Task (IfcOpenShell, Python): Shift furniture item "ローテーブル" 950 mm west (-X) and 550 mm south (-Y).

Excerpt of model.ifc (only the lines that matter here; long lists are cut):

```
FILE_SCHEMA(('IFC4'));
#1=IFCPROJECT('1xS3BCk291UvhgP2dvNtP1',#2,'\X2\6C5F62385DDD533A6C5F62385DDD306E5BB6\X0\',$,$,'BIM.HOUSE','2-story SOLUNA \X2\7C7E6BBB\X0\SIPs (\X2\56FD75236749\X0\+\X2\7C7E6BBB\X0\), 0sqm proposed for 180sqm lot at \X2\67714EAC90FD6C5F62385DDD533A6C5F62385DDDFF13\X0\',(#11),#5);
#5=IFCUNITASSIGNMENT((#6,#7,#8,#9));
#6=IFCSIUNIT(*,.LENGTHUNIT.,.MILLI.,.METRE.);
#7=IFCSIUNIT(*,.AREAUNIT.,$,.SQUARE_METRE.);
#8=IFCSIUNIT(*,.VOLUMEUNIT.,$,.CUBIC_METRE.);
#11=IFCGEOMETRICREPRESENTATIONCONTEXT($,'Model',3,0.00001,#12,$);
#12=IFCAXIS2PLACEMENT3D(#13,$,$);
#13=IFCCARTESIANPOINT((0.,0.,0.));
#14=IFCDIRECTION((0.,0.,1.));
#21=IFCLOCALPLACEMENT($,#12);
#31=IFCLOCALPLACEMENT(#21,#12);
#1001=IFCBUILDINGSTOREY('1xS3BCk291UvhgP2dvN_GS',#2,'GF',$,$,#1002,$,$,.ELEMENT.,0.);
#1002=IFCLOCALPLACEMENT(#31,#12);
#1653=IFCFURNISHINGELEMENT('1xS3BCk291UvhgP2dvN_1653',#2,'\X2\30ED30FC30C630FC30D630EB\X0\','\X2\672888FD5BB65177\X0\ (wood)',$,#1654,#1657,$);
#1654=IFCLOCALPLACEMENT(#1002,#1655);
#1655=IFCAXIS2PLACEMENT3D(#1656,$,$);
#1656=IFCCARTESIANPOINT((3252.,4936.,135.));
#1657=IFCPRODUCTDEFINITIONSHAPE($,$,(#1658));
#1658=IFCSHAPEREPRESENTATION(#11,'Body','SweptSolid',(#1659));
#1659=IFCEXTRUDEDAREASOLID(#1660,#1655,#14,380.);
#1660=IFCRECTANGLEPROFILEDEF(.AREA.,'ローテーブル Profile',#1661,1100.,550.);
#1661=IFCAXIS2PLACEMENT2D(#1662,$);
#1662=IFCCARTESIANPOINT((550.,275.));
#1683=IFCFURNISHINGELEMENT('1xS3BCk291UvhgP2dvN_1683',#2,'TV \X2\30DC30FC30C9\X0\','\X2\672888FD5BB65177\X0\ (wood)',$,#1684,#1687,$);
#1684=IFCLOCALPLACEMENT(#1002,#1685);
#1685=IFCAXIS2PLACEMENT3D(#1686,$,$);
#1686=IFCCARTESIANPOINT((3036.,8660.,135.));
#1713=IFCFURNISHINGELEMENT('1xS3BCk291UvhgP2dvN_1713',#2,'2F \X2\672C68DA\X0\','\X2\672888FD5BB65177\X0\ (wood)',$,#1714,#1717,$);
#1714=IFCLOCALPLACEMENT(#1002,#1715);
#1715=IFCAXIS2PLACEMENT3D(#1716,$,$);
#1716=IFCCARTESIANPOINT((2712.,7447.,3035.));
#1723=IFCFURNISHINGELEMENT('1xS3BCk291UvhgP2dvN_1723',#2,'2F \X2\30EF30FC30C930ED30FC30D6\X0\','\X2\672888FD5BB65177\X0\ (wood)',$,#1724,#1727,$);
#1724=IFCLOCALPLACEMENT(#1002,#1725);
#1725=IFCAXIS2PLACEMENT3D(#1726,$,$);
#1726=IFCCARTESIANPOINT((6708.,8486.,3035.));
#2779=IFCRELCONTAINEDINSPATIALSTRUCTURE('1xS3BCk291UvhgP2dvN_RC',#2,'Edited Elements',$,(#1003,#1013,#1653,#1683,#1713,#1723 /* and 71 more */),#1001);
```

```python
import ifcopenshell
import ifcopenshell.api.geometry
import ifcopenshell.util.placement
import ifcopenshell.util.unit

model = ifcopenshell.open("model.ifc")
unit_scale = ifcopenshell.util.unit.calculate_unit_scale(model)

item = model.by_guid("1xS3BCk291UvhgP2dvN_1653")
matrix = ifcopenshell.util.placement.get_local_placement(item.ObjectPlacement)
matrix[0, 3] -= 0.95 / unit_scale
matrix[1, 3] -= 0.55 / unit_scale
ifcopenshell.api.geometry.edit_object_placement(model, product=item, matrix=matrix, is_si=False)

print(ifcopenshell.util.placement.get_local_placement(item.ObjectPlacement).round(3) + 0.0)

model.write("model_v2.ifc")
```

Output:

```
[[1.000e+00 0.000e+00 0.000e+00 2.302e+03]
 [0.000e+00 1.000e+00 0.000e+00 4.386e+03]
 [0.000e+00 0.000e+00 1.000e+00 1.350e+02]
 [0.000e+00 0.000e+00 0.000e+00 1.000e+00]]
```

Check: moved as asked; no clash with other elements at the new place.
